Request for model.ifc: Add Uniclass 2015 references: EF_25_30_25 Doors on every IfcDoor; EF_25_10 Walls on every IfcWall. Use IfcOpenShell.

First a look at what the model holds.

```python
import ifcopenshell

model = ifcopenshell.open("model.ifc")
print(model.schema)
print("classifications:", [c.Name for c in model.by_type("IfcClassification")])
for ifc_class in ("IfcDoor", "IfcRoof", "IfcStair", "IfcWall", "IfcWindow"):
    print(ifc_class, len(model.by_type(ifc_class)))
```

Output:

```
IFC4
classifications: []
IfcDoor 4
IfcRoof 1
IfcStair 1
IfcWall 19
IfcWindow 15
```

```python
import ifcopenshell
import ifcopenshell.api.classification

model = ifcopenshell.open("model.ifc")

system = ifcopenshell.api.classification.add_classification(model, classification="Uniclass 2015")

codes = {
    "IfcDoor": ("EF_25_30_25", "Doors"),
    "IfcWall": ("EF_25_10", "Walls"),
}
for ifc_class, (code, name) in codes.items():
    products = model.by_type(ifc_class)
    ifcopenshell.api.classification.add_reference(
        model, products=products, classification=system, identification=code, name=name
    )
    print(code, len(products))

model.write("model_updated.ifc")
```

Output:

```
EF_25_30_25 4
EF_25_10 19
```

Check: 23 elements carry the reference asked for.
